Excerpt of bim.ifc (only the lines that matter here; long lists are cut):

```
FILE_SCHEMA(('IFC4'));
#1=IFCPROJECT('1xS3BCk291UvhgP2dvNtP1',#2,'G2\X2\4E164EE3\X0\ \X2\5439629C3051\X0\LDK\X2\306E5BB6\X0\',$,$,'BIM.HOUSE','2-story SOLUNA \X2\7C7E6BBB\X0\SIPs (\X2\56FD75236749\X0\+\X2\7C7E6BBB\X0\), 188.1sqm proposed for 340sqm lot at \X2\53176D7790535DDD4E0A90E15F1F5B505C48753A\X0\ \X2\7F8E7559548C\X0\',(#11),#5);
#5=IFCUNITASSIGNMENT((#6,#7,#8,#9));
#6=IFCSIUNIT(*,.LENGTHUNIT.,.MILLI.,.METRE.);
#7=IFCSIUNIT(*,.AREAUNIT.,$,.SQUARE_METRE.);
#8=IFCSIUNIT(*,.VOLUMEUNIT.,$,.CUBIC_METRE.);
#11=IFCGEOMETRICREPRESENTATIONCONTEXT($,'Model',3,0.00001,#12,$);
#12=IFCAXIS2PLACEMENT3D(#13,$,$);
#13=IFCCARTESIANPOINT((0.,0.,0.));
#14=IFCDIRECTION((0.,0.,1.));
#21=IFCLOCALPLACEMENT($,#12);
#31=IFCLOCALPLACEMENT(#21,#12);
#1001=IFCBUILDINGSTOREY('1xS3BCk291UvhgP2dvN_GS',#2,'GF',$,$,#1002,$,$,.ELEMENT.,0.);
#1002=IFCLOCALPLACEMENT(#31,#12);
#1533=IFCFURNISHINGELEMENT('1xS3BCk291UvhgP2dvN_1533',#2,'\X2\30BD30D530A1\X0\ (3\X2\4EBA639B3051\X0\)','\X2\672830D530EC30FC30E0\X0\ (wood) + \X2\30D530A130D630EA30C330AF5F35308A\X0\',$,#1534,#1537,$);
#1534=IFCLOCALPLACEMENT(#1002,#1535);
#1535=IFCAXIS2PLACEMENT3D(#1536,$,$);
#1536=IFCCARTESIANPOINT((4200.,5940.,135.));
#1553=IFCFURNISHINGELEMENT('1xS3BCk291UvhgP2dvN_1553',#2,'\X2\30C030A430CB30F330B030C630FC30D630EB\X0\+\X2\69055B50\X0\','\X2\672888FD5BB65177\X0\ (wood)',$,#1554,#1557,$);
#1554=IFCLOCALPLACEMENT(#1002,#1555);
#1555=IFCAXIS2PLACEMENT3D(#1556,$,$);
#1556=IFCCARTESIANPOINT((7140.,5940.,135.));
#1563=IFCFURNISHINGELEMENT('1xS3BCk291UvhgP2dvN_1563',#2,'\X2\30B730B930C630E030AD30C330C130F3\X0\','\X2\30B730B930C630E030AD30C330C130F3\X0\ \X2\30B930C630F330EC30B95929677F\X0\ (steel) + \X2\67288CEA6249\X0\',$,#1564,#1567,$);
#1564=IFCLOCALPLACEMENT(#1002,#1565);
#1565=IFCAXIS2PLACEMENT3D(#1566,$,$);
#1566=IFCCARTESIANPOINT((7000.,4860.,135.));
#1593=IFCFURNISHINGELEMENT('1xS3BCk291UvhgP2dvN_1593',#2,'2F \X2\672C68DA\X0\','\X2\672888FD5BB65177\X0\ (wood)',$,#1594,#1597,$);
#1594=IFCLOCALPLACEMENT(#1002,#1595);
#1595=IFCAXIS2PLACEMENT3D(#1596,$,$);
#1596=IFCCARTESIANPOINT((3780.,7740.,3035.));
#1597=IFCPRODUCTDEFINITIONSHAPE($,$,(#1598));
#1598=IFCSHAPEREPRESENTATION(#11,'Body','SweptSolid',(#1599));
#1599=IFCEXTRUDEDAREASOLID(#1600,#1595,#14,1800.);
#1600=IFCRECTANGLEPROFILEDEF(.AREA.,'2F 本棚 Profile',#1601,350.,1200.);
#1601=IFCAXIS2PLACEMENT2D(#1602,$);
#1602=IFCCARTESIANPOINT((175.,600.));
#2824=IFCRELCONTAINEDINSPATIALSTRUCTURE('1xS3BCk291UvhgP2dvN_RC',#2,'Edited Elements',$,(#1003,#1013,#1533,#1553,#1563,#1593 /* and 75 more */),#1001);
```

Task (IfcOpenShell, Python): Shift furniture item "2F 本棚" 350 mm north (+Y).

```python
import ifcopenshell
import ifcopenshell.api.geometry
import ifcopenshell.util.placement
import ifcopenshell.util.unit

model = ifcopenshell.open("bim.ifc")
unit_scale = ifcopenshell.util.unit.calculate_unit_scale(model)

item = model.by_guid("1xS3BCk291UvhgP2dvN_1593")
matrix = ifcopenshell.util.placement.get_local_placement(item.ObjectPlacement)
matrix[1, 3] += 0.35 / unit_scale
ifcopenshell.api.geometry.edit_object_placement(model, product=item, matrix=matrix, is_si=False)

print(ifcopenshell.util.placement.get_local_placement(item.ObjectPlacement).round(3) + 0.0)

model.write("bim_v2.ifc")
```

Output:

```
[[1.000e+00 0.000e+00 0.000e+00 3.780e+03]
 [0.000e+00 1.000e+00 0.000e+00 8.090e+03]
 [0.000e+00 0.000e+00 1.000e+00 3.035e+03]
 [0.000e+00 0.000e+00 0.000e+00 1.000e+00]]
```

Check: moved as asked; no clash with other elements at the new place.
